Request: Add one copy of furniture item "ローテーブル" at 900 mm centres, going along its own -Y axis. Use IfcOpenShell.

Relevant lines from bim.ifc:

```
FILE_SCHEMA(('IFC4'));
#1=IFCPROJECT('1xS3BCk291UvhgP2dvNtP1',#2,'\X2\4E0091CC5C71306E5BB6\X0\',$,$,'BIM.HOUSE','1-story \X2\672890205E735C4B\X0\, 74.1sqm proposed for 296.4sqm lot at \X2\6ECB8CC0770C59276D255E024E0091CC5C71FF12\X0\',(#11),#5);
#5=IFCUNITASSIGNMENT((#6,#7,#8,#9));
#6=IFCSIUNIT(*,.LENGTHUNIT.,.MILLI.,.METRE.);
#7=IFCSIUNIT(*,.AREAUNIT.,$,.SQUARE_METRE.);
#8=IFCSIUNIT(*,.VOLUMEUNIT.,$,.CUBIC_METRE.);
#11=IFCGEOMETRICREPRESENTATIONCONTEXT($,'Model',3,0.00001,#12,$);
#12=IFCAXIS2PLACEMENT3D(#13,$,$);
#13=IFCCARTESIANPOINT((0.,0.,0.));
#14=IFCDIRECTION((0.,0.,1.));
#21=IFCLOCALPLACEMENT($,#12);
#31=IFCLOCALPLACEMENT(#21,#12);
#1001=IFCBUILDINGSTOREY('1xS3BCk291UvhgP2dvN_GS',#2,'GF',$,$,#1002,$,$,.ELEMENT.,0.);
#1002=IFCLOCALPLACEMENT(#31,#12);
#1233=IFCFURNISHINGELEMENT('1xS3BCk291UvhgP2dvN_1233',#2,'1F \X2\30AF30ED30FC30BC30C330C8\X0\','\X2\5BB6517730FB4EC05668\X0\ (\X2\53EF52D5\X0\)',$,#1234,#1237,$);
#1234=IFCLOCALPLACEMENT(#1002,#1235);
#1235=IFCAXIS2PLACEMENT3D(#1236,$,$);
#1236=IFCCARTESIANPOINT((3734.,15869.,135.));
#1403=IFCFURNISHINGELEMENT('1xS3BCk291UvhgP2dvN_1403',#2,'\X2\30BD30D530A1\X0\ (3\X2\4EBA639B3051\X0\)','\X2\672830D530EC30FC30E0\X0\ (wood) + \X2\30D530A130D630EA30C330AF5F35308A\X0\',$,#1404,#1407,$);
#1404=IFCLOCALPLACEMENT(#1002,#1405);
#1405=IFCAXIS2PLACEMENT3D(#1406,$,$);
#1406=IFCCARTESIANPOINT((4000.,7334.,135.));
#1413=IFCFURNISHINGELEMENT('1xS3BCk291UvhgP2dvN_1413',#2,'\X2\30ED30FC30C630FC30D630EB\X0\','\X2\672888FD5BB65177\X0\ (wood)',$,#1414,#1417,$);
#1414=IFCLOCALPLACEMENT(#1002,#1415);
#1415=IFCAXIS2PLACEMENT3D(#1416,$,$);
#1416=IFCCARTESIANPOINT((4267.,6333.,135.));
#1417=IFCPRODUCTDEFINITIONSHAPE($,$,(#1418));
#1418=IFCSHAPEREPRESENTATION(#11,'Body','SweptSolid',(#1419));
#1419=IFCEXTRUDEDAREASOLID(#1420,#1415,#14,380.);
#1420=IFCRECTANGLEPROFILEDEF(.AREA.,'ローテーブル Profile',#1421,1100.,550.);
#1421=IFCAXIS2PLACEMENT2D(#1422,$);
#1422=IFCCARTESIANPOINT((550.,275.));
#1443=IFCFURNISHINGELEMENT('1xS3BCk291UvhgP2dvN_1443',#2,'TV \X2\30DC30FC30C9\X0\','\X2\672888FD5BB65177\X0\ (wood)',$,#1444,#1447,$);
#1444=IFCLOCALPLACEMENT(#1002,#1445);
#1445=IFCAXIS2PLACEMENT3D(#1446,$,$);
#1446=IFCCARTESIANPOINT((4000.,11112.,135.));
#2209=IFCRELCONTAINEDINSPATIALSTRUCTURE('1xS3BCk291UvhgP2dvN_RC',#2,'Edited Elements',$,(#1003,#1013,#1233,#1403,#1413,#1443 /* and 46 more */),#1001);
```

```python
import ifcopenshell
import ifcopenshell.api.geometry
import ifcopenshell.api.root
import ifcopenshell.util.element
import ifcopenshell.util.placement

model = ifcopenshell.open("bim.ifc")


def reuse_history(source, copy):
    """copy_class also copies each property set's owner history, people and application; keep the originals."""
    for rel in copy.IsDefinedBy:
        if rel.is_a("IfcRelDefinesByProperties") and (history := rel.RelatingPropertyDefinition.OwnerHistory):
            rel.RelatingPropertyDefinition.OwnerHistory = source.OwnerHistory
            ifcopenshell.util.element.remove_deep2(model, history)


source = model.by_guid("1xS3BCk291UvhgP2dvN_1413")
base = ifcopenshell.util.placement.get_local_placement(source.ObjectPlacement)
step = -base[:3, 1] * 900.0

for i in range(1, 2):
    copy = ifcopenshell.api.root.copy_class(model, product=source)
    copy.Representation = ifcopenshell.util.element.copy_deep(
        model, source.Representation, exclude=["IfcGeometricRepresentationContext", "IfcRepresentationMap"]
    )
    reuse_history(source, copy)
    matrix = base.copy()
    matrix[:3, 3] += i * step
    print("added at", matrix[:3, 3].round(3) + 0.0)
    ifcopenshell.api.geometry.edit_object_placement(model, product=copy, matrix=matrix, is_si=False)

model.write("bim-out.ifc")
```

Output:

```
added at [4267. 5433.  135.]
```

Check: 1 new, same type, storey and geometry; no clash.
